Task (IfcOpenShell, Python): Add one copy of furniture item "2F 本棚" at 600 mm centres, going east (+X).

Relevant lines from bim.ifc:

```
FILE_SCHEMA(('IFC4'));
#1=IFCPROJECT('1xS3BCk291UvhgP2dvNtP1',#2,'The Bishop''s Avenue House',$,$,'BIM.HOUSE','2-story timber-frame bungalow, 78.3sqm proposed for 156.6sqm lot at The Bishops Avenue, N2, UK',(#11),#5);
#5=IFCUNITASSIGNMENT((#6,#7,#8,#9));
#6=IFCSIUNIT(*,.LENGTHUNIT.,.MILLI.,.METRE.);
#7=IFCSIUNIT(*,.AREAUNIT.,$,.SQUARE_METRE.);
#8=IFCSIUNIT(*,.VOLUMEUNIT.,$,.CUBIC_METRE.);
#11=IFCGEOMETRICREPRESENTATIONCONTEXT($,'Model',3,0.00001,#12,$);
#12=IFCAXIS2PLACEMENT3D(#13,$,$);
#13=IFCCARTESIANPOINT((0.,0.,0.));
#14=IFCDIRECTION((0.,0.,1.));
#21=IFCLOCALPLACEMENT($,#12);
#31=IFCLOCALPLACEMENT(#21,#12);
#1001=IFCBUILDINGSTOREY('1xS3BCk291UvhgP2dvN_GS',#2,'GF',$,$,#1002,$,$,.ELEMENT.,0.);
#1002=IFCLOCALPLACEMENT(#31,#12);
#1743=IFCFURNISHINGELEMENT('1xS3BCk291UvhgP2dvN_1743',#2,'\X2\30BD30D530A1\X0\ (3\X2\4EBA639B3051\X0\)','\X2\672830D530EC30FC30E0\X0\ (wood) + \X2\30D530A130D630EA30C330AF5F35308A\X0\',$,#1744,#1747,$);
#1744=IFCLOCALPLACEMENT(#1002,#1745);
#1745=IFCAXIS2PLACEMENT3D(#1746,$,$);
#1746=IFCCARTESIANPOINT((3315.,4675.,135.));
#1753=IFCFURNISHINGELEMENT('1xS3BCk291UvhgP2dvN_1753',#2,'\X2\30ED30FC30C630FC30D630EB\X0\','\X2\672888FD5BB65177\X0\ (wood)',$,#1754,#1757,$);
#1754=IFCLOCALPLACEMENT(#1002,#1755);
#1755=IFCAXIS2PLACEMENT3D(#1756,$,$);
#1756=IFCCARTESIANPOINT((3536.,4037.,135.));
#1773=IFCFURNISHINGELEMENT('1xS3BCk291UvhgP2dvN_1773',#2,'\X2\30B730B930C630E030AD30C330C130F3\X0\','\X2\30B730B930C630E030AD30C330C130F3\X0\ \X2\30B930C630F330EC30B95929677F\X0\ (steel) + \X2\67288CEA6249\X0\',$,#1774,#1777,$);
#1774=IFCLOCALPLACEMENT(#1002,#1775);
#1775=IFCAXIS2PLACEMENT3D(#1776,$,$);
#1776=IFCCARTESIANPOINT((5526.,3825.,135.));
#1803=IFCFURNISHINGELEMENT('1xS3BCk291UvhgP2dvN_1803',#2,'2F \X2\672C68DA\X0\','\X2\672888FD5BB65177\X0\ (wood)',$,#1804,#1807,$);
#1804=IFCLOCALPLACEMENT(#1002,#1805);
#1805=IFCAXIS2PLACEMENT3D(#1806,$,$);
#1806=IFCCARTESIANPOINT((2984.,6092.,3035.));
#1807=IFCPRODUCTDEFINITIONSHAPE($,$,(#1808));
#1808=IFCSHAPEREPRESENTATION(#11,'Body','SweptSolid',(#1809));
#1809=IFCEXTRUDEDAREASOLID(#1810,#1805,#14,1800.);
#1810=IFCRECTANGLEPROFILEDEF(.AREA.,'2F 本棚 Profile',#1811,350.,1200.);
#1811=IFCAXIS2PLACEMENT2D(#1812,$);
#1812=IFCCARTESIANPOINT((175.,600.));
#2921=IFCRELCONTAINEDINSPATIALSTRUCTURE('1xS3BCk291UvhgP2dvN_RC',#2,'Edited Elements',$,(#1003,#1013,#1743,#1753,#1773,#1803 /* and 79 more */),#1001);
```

```python
import numpy as np
import ifcopenshell
import ifcopenshell.api.geometry
import ifcopenshell.api.root
import ifcopenshell.util.element
import ifcopenshell.util.placement
import ifcopenshell.util.unit

model = ifcopenshell.open("bim.ifc")
unit_scale = ifcopenshell.util.unit.calculate_unit_scale(model)


def reuse_history(source, copy):
    """copy_class also copies each property set's owner history, people and application; keep the originals."""
    for rel in copy.IsDefinedBy:
        if rel.is_a("IfcRelDefinesByProperties") and (history := rel.RelatingPropertyDefinition.OwnerHistory):
            rel.RelatingPropertyDefinition.OwnerHistory = source.OwnerHistory
            ifcopenshell.util.element.remove_deep2(model, history)


source = model.by_id(1803)
base = ifcopenshell.util.placement.get_local_placement(source.ObjectPlacement)
step = np.array([1.0, 0.0, 0.0]) * 0.6 / unit_scale

for i in range(1, 2):
    copy = ifcopenshell.api.root.copy_class(model, product=source)
    copy.Representation = ifcopenshell.util.element.copy_deep(
        model, source.Representation, exclude=["IfcGeometricRepresentationContext", "IfcRepresentationMap"]
    )
    reuse_history(source, copy)
    matrix = base.copy()
    matrix[:3, 3] += i * step
    print("added at", matrix[:3, 3].round(3) + 0.0)
    ifcopenshell.api.geometry.edit_object_placement(model, product=copy, matrix=matrix, is_si=False)

model.write("bim_v2.ifc")
```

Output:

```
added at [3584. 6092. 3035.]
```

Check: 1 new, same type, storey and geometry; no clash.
